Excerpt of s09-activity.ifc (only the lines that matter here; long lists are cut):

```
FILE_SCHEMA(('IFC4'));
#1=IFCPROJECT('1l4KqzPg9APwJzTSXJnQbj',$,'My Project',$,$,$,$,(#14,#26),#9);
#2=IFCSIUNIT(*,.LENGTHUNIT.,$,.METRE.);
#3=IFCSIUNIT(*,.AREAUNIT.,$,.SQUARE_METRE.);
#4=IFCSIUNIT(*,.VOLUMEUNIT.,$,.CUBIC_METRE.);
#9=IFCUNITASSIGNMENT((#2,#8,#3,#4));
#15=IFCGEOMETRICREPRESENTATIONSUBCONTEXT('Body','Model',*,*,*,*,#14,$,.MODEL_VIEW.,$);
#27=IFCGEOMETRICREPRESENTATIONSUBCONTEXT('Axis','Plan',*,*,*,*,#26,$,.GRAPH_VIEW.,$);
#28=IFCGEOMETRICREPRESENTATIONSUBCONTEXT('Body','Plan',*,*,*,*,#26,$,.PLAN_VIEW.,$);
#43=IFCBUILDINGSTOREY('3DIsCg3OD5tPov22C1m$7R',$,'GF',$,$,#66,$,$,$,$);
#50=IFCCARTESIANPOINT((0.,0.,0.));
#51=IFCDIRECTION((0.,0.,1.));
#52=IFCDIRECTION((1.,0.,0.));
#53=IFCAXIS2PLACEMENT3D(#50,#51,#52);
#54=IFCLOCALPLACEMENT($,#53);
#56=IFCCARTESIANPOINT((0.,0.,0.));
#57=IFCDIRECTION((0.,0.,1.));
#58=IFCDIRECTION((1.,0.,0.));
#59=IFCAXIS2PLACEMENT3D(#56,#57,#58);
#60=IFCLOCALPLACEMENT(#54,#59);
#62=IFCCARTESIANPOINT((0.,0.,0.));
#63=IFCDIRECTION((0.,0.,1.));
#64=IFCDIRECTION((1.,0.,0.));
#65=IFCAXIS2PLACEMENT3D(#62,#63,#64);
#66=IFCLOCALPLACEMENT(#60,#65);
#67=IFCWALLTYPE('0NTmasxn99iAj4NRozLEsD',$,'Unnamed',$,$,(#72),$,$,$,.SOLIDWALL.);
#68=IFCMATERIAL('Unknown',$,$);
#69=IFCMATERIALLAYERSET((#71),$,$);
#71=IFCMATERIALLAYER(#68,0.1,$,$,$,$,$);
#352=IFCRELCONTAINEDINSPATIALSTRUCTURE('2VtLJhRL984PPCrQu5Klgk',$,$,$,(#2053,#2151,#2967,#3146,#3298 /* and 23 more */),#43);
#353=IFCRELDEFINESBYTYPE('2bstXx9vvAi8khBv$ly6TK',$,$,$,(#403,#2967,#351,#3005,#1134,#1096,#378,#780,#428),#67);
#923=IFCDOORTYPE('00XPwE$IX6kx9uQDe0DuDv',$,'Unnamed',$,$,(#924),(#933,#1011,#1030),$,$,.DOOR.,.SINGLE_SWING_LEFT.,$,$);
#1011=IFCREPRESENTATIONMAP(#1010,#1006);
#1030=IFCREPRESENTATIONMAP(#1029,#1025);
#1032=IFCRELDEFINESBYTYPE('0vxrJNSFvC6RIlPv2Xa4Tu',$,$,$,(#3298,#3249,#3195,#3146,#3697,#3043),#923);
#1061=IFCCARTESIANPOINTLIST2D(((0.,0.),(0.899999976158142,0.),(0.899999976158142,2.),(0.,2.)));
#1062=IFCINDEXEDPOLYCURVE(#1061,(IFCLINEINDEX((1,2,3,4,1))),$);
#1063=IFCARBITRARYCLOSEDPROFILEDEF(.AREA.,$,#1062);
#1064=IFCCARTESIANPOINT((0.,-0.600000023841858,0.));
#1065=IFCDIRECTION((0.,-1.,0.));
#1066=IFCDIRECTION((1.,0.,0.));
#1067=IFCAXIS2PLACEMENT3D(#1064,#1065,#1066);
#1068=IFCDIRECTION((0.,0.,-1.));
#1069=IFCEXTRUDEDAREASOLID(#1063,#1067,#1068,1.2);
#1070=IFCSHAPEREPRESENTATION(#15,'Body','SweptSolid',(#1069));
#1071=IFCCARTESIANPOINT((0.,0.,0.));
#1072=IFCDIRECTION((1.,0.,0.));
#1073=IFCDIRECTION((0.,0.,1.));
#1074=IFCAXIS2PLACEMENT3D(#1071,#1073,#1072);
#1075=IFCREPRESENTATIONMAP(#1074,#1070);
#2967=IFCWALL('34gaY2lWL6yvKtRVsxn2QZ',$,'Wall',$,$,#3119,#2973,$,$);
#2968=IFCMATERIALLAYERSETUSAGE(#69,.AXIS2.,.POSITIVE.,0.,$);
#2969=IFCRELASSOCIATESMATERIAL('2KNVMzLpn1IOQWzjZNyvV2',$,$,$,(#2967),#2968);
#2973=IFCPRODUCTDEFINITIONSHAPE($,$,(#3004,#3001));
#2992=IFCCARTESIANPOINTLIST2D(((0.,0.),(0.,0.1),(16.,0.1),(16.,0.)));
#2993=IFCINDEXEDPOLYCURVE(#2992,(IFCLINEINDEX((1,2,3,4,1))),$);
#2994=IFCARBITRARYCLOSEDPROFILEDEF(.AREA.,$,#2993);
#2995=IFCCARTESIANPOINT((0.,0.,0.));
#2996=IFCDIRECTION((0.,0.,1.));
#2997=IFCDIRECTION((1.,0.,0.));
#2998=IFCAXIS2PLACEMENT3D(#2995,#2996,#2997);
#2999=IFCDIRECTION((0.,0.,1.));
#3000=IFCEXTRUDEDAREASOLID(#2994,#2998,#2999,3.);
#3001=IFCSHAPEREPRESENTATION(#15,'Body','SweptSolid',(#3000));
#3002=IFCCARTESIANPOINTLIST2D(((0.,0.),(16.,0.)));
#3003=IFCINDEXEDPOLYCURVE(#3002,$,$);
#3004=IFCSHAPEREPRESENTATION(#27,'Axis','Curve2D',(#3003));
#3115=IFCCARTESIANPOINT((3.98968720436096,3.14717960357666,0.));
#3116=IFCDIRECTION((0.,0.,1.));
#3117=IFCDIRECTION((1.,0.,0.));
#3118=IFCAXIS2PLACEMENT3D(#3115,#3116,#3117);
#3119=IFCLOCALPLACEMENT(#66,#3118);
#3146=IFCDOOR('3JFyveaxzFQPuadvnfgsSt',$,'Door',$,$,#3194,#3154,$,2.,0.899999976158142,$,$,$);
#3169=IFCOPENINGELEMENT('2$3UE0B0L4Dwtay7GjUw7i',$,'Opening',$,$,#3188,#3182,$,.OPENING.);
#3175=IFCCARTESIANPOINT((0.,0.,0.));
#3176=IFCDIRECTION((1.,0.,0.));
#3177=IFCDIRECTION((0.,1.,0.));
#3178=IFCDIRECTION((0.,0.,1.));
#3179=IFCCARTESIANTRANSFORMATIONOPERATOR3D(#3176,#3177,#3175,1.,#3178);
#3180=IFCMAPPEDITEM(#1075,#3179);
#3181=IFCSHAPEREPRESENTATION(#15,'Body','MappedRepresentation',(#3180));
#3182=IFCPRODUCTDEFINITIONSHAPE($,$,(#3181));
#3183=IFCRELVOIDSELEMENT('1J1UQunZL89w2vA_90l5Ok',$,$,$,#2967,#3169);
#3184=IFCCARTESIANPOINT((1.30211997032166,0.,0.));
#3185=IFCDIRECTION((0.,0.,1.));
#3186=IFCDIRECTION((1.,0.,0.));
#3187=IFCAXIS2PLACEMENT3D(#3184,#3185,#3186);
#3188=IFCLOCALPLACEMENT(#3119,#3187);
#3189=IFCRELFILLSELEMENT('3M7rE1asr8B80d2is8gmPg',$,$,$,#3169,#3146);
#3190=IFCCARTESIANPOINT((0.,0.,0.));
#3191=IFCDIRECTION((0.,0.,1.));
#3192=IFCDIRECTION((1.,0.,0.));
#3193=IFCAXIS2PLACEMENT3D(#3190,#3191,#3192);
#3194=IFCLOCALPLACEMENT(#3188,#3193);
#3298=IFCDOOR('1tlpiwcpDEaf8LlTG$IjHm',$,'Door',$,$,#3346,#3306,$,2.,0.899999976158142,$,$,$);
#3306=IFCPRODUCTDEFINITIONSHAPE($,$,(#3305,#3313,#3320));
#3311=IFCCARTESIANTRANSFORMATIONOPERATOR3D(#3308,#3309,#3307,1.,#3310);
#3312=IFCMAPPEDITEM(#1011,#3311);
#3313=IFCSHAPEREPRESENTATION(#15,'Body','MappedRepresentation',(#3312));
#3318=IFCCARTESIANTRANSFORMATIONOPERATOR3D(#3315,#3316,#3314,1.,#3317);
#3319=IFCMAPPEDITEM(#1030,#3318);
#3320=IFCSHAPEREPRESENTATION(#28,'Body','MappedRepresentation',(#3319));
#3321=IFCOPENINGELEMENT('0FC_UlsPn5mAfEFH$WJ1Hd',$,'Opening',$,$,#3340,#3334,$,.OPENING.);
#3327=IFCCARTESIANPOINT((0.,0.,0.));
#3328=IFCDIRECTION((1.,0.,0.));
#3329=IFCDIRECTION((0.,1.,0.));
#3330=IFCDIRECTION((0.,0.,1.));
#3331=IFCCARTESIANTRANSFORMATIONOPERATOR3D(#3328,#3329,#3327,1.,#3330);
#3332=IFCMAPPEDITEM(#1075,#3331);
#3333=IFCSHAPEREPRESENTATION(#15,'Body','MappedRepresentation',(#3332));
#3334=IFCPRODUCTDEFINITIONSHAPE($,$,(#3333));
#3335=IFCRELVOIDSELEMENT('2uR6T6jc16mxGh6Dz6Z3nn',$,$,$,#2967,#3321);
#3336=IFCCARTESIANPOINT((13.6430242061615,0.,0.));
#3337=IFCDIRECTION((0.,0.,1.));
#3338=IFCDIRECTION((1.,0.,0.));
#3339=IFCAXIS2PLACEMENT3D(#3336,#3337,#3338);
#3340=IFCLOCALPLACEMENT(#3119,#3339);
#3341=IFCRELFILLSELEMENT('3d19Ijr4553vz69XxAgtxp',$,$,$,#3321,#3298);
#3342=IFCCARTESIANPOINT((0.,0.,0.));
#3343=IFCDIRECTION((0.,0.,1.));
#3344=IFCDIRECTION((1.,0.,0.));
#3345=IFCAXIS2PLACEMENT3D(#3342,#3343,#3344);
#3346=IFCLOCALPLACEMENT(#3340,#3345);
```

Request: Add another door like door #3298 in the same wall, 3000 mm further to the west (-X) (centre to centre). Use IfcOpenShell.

```python
import ifcopenshell
import ifcopenshell.api.feature
import ifcopenshell.api.geometry
import ifcopenshell.api.root
import ifcopenshell.geom
import ifcopenshell.util.element
import ifcopenshell.util.placement
import ifcopenshell.util.shape
import ifcopenshell.util.unit

model = ifcopenshell.open("s09-activity.ifc")
unit_scale = ifcopenshell.util.unit.calculate_unit_scale(model)
settings = ifcopenshell.geom.settings()


def volume(element):
    """Net volume in cubic metres, openings subtracted."""
    shape = ifcopenshell.geom.create_shape(settings, element)
    return ifcopenshell.util.shape.get_volume(shape.geometry)


door = model.by_guid("1tlpiwcpDEaf8LlTG$IjHm")
opening = door.FillsVoids[0].RelatingOpeningElement
wall = opening.VoidsElements[0].RelatingBuildingElement
before = volume(wall)
shift = ifcopenshell.util.placement.get_local_placement(wall.ObjectPlacement)[:3, 0] * -3 / unit_scale

# copy_class copies the void relationship, type, container and properties, but no geometry.
new_opening = ifcopenshell.api.root.copy_class(model, product=opening)
new_opening.Representation = ifcopenshell.util.element.copy_deep(
    model, opening.Representation, exclude=["IfcGeometricRepresentationContext", "IfcRepresentationMap"]
)
new_door = ifcopenshell.api.root.copy_class(model, product=door)
new_door.Representation = ifcopenshell.util.element.copy_deep(
    model, door.Representation, exclude=["IfcGeometricRepresentationContext", "IfcRepresentationMap"]
)
ifcopenshell.api.feature.add_filling(model, opening=new_opening, element=new_door)

for old, new in ((opening, new_opening), (door, new_door)):
    matrix = ifcopenshell.util.placement.get_local_placement(old.ObjectPlacement)
    matrix[:3, 3] += shift
    ifcopenshell.api.geometry.edit_object_placement(model, product=new, matrix=matrix, is_si=False)

after = volume(wall)

print(f"wall volume {before:.3f} -> {after:.3f} m3")

model.write("s09-activity_updated.ifc")
```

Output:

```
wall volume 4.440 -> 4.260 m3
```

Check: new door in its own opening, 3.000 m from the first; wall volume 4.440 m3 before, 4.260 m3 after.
